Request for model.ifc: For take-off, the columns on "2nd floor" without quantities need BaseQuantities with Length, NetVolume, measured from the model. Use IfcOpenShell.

First a look at what the model holds.

```python
import ifcopenshell
import ifcopenshell.util.element
import ifcopenshell.util.unit

model = ifcopenshell.open("model.ifc")
print(model.schema)
for unit_type in ("LENGTHUNIT", "AREAUNIT", "VOLUMEUNIT"):
    print(unit_type, ifcopenshell.util.unit.calculate_unit_scale(model, unit_type))
storey = next(s for s in model.by_type("IfcBuildingStorey") if s.Name == "2nd floor")
columns = [e for e in ifcopenshell.util.element.get_decomposition(storey) if e.is_a("IfcColumn")]
for e in sorted(columns, key=lambda e: e.id()):
    print(e.id(), e.is_a(), e.Name, list(ifcopenshell.util.element.get_psets(e, qtos_only=True)), sep=" | ")
```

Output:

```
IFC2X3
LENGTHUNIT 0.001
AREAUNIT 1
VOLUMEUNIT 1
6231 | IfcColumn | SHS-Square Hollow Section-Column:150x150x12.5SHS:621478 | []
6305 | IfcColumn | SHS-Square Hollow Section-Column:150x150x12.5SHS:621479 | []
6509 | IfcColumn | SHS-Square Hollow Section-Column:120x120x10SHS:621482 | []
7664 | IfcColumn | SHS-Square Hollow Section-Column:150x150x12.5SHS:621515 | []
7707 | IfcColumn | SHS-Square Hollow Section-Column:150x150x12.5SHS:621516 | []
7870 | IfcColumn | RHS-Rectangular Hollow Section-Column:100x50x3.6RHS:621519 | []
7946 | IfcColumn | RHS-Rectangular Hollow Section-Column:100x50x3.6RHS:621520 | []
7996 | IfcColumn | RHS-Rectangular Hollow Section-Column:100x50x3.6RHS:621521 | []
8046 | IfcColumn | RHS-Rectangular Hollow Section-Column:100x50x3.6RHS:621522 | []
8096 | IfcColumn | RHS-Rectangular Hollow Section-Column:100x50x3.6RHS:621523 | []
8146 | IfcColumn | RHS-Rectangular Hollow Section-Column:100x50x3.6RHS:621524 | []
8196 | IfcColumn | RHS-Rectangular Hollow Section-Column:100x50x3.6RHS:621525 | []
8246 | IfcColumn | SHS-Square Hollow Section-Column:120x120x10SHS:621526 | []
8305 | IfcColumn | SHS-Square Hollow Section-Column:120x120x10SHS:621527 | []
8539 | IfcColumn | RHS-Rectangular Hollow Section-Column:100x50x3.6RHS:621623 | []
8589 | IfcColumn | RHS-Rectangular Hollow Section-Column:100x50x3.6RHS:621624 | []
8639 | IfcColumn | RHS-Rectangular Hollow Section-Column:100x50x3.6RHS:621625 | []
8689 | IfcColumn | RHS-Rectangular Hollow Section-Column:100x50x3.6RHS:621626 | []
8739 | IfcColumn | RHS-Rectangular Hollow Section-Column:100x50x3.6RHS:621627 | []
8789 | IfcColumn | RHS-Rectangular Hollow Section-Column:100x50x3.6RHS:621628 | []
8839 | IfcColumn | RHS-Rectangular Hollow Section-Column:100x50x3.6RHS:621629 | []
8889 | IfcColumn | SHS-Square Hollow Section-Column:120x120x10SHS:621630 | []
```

```python
import ifcopenshell
import ifcopenshell.api.pset
import ifcopenshell.geom
import ifcopenshell.util.element
import ifcopenshell.util.shape
import ifcopenshell.util.unit

model = ifcopenshell.open("model.ifc")
unit_scale = ifcopenshell.util.unit.calculate_unit_scale(model)
volume_scale = ifcopenshell.util.unit.calculate_unit_scale(model, "VOLUMEUNIT")
settings = ifcopenshell.geom.settings()

storey = next(s for s in model.by_type("IfcBuildingStorey") if s.Name == "2nd floor")
columns = [e for e in ifcopenshell.util.element.get_decomposition(storey) if e.is_a("IfcColumn")]

for e in sorted(columns, key=lambda e: e.id()):
    if ifcopenshell.util.element.get_psets(e, qtos_only=True, should_inherit=False):
        continue
    # Geometry comes back in metres, in the element's own axes.
    shape = ifcopenshell.geom.create_shape(settings, e)
    values = {
        "Length": ifcopenshell.util.shape.get_z(shape.geometry) / unit_scale,
        "NetVolume": ifcopenshell.util.shape.get_volume(shape.geometry) / volume_scale,
    }
    qto = ifcopenshell.api.pset.add_qto(model, product=e, name="BaseQuantities")
    ifcopenshell.api.pset.edit_qto(model, qto=qto, properties=values)
    print(e.id(), {k: round(v, 3) for k, v in values.items()})

model.write("model-out.ifc")
```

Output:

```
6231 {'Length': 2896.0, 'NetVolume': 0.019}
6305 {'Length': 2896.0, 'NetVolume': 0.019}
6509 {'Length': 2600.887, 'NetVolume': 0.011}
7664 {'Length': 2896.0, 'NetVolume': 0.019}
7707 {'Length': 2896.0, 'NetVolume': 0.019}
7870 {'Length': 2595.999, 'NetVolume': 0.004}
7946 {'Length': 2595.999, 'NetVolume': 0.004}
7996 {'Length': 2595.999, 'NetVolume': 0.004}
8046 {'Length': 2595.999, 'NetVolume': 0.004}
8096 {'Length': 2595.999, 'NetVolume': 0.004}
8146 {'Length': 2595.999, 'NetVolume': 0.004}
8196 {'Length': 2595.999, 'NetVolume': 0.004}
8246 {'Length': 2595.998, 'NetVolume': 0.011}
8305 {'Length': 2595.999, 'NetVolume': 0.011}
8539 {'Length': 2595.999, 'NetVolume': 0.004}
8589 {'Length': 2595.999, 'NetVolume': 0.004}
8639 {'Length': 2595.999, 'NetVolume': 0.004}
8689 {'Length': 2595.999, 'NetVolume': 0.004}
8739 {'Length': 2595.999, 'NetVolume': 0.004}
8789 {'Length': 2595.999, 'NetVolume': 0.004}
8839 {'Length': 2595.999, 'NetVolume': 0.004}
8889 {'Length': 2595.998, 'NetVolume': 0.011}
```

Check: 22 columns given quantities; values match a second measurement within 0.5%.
